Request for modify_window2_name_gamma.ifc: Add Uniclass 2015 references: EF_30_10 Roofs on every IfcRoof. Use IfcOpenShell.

First a look at what the model holds.

```python
import ifcopenshell

model = ifcopenshell.open("modify_window2_name_gamma.ifc")
print(model.schema)
print("classifications:", [c.Name for c in model.by_type("IfcClassification")])
for ifc_class in ("IfcDoor", "IfcRoof", "IfcStair", "IfcWall", "IfcWindow"):
    print(ifc_class, len(model.by_type(ifc_class)))
```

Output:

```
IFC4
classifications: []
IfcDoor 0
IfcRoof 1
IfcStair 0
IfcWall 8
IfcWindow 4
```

```python
import ifcopenshell
import ifcopenshell.api.classification

model = ifcopenshell.open("modify_window2_name_gamma.ifc")

system = ifcopenshell.api.classification.add_classification(model, classification="Uniclass 2015")

codes = {
    "IfcRoof": ("EF_30_10", "Roofs"),
}
for ifc_class, (code, name) in codes.items():
    products = model.by_type(ifc_class)
    ifcopenshell.api.classification.add_reference(
        model, products=products, classification=system, identification=code, name=name
    )
    print(code, len(products))

model.write("modify_window2_name_gamma_edited.ifc")
```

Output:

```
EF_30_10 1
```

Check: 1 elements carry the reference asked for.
